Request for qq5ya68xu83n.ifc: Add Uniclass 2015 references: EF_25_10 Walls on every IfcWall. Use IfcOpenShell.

First a look at what the model holds.

```python
import ifcopenshell

model = ifcopenshell.open("qq5ya68xu83n.ifc")
print(model.schema)
print("classifications:", [c.Name for c in model.by_type("IfcClassification")])
for ifc_class in ("IfcDoor", "IfcRoof", "IfcStair", "IfcWall", "IfcWindow"):
    print(ifc_class, len(model.by_type(ifc_class)))
```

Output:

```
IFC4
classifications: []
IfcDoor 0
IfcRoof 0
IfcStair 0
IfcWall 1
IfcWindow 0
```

```python
import ifcopenshell
import ifcopenshell.api.classification

model = ifcopenshell.open("qq5ya68xu83n.ifc")

system = ifcopenshell.api.classification.add_classification(model, classification="Uniclass 2015")

codes = {
    "IfcWall": ("EF_25_10", "Walls"),
}
for ifc_class, (code, name) in codes.items():
    products = model.by_type(ifc_class)
    ifcopenshell.api.classification.add_reference(
        model, products=products, classification=system, identification=code, name=name
    )
    print(code, len(products))

model.write("qq5ya68xu83n-out.ifc")
```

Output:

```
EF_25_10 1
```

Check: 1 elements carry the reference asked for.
